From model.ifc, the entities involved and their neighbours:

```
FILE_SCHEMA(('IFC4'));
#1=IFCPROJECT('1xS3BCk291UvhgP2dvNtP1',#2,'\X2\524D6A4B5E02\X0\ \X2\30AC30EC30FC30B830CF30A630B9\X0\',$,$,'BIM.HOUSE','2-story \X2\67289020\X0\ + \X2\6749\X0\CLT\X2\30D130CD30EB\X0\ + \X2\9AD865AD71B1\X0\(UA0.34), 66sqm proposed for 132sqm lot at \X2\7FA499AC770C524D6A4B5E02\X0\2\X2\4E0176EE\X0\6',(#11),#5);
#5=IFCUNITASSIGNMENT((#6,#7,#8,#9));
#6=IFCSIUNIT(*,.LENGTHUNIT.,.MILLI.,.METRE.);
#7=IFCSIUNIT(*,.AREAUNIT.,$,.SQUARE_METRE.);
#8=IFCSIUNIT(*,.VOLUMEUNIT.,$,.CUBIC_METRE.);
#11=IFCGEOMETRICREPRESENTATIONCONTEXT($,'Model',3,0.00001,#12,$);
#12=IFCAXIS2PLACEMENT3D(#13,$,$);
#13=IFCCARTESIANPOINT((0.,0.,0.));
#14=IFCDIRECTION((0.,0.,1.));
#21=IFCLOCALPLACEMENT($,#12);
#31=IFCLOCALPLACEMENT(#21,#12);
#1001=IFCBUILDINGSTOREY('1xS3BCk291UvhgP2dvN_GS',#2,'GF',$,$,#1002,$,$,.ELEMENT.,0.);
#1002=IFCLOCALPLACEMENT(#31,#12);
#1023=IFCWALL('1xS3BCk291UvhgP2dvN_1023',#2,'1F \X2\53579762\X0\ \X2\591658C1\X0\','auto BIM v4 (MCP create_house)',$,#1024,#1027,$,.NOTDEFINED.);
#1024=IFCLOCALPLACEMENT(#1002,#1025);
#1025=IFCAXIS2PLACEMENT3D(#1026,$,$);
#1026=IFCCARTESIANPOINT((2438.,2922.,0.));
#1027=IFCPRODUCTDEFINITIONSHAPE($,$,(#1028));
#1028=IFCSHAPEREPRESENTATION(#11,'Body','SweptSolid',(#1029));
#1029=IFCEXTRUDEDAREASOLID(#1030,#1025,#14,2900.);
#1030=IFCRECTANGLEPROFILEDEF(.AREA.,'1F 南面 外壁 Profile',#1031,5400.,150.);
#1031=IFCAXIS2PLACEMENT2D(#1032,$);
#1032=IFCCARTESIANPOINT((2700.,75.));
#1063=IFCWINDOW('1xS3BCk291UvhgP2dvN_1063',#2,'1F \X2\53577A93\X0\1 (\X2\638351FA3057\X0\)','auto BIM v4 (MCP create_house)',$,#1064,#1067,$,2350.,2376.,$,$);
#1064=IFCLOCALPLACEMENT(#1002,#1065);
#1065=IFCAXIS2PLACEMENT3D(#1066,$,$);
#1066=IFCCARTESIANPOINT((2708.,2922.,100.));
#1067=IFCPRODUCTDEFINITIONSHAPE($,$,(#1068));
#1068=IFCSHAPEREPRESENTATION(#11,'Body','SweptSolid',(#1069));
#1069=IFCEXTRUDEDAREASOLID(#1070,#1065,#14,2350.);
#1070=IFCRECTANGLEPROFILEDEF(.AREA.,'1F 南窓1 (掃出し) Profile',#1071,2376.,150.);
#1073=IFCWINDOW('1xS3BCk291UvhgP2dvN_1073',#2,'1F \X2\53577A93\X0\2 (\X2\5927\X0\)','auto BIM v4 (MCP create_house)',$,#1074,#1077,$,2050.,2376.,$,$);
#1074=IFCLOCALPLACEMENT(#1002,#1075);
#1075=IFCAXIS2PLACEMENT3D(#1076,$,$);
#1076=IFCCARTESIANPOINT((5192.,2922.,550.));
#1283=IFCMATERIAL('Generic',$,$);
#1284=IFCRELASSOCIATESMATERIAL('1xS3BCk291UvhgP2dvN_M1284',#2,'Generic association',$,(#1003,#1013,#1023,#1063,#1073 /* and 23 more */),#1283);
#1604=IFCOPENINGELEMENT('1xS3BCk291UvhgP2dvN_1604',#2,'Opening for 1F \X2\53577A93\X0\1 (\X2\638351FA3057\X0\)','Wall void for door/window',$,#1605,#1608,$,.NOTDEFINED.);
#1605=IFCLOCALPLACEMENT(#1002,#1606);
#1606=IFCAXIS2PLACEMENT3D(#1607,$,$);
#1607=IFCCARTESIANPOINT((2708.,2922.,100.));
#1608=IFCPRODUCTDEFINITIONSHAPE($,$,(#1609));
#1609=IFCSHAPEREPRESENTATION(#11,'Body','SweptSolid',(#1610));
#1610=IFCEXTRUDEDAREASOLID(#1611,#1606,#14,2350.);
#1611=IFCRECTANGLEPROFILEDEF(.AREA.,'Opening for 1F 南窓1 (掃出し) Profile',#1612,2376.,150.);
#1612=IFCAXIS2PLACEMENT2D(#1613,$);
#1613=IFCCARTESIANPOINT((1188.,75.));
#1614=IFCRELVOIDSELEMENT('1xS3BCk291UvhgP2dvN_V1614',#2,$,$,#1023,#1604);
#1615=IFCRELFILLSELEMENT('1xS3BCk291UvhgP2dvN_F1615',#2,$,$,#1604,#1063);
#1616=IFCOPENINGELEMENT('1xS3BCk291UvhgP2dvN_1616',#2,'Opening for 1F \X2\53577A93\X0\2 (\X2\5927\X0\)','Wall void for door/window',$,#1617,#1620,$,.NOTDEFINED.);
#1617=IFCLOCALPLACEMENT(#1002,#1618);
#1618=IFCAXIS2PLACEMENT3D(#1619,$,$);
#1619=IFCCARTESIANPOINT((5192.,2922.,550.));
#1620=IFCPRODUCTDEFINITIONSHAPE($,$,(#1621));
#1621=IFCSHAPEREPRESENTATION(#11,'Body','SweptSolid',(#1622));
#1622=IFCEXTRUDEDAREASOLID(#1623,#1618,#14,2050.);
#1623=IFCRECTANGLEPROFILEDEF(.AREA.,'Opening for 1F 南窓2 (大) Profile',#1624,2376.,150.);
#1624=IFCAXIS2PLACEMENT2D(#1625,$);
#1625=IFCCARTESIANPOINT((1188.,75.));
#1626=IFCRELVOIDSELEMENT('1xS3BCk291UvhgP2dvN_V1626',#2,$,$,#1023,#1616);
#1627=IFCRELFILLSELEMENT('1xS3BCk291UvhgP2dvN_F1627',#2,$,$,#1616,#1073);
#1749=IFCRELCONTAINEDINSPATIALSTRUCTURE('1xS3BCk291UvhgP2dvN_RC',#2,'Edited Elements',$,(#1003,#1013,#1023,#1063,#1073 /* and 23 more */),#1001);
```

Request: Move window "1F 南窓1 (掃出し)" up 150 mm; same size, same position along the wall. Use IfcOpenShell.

```python
import numpy as np
import ifcopenshell
import ifcopenshell.api.geometry
import ifcopenshell.util.placement
import ifcopenshell.util.unit

model = ifcopenshell.open("model.ifc")
unit_scale = ifcopenshell.util.unit.calculate_unit_scale(model)

window = model.by_guid("1xS3BCk291UvhgP2dvN_1063")
opening = window.FillsVoids[0].RelatingOpeningElement
dz = 150.0

shift = np.array([0.0, 0.0, dz])
# The window is not placed relative to its opening, so move both.
for product in (opening, window):
    matrix = ifcopenshell.util.placement.get_local_placement(product.ObjectPlacement)
    matrix[:3, 3] += shift
    ifcopenshell.api.geometry.edit_object_placement(model, product=product, matrix=matrix, is_si=False)

print(f"moved by {dz * unit_scale:+.3f} m")

model.write("model_edited.ifc")
```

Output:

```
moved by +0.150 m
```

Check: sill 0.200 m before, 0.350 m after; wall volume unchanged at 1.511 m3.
